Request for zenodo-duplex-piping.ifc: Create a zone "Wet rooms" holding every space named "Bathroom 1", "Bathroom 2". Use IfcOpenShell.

First a look at what the model holds.

```python
import ifcopenshell

model = ifcopenshell.open("zenodo-duplex-piping.ifc")
print(model.schema)
seen = {}
for space in model.by_type("IfcSpace"):
    seen[space.LongName] = seen.get(space.LongName, 0) + 1
for name, count in sorted(seen.items(), key=str):
    print(count, "x", name)
print("zones:", [z.Name for z in model.by_type("IfcZone")][:20])
```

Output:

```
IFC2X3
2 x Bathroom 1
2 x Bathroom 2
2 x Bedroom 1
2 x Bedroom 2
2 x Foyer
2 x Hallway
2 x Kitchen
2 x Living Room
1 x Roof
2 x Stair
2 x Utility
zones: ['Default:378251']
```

```python
import ifcopenshell
import ifcopenshell.api.group
import ifcopenshell.api.root

model = ifcopenshell.open("zenodo-duplex-piping.ifc")

names = {"Bathroom 1", "Bathroom 2"}
spaces = [s for s in model.by_type("IfcSpace") if s.LongName in names]

zone = ifcopenshell.api.root.create_entity(model, ifc_class="IfcZone", name="Wet rooms")
ifcopenshell.api.group.assign_group(model, products=spaces, group=zone)
print(len(spaces), "spaces in", zone.Name)

model.write("zenodo-duplex-piping_edited.ifc")
```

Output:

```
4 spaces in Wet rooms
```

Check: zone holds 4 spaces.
